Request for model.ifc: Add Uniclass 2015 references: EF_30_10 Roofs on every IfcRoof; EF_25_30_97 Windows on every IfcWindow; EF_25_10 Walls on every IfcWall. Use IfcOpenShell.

First a look at what the model holds.

```python
import ifcopenshell

model = ifcopenshell.open("model.ifc")
print(model.schema)
print("classifications:", [c.Name for c in model.by_type("IfcClassification")])
for ifc_class in ("IfcDoor", "IfcRoof", "IfcStair", "IfcWall", "IfcWindow"):
    print(ifc_class, len(model.by_type(ifc_class)))
```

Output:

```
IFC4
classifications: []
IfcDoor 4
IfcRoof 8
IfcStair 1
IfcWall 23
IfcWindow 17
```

```python
import ifcopenshell
import ifcopenshell.api.classification

model = ifcopenshell.open("model.ifc")

system = ifcopenshell.api.classification.add_classification(model, classification="Uniclass 2015")

codes = {
    "IfcRoof": ("EF_30_10", "Roofs"),
    "IfcWindow": ("EF_25_30_97", "Windows"),
    "IfcWall": ("EF_25_10", "Walls"),
}
for ifc_class, (code, name) in codes.items():
    products = model.by_type(ifc_class)
    ifcopenshell.api.classification.add_reference(
        model, products=products, classification=system, identification=code, name=name
    )
    print(code, len(products))

model.write("model_updated.ifc")
```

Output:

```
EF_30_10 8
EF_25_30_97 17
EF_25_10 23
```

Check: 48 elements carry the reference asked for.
